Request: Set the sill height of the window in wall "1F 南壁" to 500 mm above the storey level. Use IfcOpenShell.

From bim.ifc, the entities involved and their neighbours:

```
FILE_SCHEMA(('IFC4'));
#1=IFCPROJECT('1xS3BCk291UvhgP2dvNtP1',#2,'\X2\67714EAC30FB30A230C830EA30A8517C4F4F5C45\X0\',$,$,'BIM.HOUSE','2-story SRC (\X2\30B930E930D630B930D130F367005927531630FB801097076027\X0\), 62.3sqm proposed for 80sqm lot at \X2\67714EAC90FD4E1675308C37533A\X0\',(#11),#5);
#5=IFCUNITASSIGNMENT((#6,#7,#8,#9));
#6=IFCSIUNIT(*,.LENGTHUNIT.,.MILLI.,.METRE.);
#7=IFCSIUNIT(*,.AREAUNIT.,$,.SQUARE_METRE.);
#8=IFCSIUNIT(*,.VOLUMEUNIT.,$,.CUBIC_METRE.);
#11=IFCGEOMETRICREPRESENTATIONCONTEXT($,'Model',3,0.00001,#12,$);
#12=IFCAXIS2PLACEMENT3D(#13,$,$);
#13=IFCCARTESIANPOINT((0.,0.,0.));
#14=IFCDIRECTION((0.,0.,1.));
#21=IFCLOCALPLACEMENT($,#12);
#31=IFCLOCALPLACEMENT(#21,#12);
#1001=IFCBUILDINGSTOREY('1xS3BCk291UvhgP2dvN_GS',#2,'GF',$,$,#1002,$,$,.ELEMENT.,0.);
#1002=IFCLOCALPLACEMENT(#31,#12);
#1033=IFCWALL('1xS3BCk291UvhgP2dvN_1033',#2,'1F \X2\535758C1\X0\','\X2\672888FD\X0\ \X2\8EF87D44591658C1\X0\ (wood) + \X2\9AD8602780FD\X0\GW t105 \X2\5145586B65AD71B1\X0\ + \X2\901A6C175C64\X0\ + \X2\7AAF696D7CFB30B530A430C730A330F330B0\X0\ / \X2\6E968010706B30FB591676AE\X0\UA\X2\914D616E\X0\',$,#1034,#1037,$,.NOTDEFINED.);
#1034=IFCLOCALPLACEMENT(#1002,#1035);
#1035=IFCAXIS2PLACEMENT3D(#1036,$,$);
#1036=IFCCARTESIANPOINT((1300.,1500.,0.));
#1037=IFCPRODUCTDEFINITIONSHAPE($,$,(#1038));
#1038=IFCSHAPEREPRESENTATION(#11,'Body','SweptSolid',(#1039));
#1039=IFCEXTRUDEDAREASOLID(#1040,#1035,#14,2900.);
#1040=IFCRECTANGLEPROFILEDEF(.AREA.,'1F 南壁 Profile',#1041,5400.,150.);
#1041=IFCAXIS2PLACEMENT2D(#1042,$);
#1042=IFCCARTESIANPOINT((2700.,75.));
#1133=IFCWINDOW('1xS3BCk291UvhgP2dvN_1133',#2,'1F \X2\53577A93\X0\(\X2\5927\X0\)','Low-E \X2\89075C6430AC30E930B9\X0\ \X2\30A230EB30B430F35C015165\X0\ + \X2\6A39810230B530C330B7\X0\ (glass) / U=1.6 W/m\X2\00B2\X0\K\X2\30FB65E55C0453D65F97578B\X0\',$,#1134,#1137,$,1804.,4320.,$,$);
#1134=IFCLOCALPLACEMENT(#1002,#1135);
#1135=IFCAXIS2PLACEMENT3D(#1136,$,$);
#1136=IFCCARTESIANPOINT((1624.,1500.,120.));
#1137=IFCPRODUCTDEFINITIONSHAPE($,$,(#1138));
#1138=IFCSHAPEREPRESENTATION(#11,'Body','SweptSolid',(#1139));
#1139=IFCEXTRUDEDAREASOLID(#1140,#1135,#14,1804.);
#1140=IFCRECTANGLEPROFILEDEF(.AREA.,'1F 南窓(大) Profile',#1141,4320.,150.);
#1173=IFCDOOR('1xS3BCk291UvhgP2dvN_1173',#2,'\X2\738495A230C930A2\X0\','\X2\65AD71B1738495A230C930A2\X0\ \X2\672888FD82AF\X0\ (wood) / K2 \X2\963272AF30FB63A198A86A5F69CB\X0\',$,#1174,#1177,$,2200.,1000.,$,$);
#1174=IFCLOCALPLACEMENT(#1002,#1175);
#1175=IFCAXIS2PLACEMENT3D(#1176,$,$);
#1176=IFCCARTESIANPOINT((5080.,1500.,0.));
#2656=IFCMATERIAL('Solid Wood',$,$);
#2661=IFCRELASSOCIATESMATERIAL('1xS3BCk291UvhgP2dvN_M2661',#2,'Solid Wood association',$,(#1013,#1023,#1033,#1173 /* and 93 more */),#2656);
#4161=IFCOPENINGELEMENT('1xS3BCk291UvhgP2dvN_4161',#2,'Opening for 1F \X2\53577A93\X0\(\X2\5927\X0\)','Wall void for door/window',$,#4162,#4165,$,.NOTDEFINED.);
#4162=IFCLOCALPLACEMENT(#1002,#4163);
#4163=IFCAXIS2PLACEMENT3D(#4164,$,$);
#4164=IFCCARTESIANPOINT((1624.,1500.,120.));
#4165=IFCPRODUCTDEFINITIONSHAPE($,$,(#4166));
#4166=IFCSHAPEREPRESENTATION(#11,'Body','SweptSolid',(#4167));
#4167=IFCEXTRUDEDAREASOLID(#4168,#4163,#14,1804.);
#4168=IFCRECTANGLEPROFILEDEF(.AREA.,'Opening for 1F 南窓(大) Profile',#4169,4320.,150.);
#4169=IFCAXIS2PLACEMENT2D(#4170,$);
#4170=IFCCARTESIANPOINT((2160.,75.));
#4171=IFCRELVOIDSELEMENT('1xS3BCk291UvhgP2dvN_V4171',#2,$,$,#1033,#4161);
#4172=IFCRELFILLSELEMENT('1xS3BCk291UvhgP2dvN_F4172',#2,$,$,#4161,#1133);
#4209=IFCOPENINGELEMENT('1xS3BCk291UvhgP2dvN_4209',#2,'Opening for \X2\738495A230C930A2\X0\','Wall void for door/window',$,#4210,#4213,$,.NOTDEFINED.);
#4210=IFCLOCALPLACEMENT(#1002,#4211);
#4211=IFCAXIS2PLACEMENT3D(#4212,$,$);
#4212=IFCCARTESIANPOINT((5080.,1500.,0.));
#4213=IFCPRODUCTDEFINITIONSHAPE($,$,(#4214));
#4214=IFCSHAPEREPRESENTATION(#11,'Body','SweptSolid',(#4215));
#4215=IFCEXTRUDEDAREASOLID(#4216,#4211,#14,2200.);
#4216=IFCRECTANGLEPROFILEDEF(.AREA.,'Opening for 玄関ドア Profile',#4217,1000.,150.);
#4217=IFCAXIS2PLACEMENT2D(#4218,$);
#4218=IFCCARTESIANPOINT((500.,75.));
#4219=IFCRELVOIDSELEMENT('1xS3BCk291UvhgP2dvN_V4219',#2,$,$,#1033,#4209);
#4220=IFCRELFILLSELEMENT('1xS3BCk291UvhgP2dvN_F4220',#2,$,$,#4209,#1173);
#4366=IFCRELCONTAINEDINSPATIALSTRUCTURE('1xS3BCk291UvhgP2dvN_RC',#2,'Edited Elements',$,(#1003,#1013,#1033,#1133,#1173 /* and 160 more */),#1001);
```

```python
import numpy as np
import ifcopenshell
import ifcopenshell.api.geometry
import ifcopenshell.geom
import ifcopenshell.util.element
import ifcopenshell.util.placement
import ifcopenshell.util.shape
import ifcopenshell.util.unit

model = ifcopenshell.open("bim.ifc")
unit_scale = ifcopenshell.util.unit.calculate_unit_scale(model)

window = model.by_id(1133)
opening = window.FillsVoids[0].RelatingOpeningElement
storey = ifcopenshell.util.element.get_container(window, ifc_class="IfcBuildingStorey")
level = ifcopenshell.util.placement.get_local_placement(storey.ObjectPlacement)[2, 3]

# The opening's origin need not be at the sill, so measure its lowest point.
shape = ifcopenshell.geom.create_shape(ifcopenshell.geom.settings(), opening)
bottom = ifcopenshell.util.shape.get_shape_bottom_elevation(shape, shape.geometry) / unit_scale
dz = level + 500.0 - bottom

shift = np.array([0.0, 0.0, dz])
# The window is not placed relative to its opening, so move both.
for product in (opening, window):
    matrix = ifcopenshell.util.placement.get_local_placement(product.ObjectPlacement)
    matrix[:3, 3] += shift
    ifcopenshell.api.geometry.edit_object_placement(model, product=product, matrix=matrix, is_si=False)

print(f"moved by {dz * unit_scale:+.3f} m")

model.write("bim_updated.ifc")
```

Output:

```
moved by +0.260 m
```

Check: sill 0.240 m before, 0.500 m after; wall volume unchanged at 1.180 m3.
